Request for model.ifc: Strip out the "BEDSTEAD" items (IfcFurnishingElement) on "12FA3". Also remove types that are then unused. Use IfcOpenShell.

First a look at what the model holds.

```python
import ifcopenshell
import ifcopenshell.util.element

model = ifcopenshell.open("model.ifc")
print(model.schema)
storey = next(s for s in model.by_type("IfcBuildingStorey") if s.Name == "12FA3")
furniture = [e for e in ifcopenshell.util.element.get_decomposition(storey) if e.is_a("IfcFurnishingElement")]
seen = {}
for e in furniture:
    element_type = ifcopenshell.util.element.get_type(e)
    name = element_type.Name if element_type not in (None, e) else None
    seen[name] = seen.get(name, 0) + 1
for name, count in sorted(seen.items(), key=str):
    print(count, "x", name)
```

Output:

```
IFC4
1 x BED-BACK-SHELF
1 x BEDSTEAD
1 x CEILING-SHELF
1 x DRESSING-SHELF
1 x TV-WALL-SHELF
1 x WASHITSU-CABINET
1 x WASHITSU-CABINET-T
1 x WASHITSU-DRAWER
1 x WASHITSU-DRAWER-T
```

```python
import ifcopenshell
import ifcopenshell.api.root
import ifcopenshell.util.element

model = ifcopenshell.open("model.ifc")

storey = next(s for s in model.by_type("IfcBuildingStorey") if s.Name == "12FA3")
furniture = [e for e in ifcopenshell.util.element.get_decomposition(storey) if e.is_a("IfcFurnishingElement")]
targets = [e for e in furniture if (t := ifcopenshell.util.element.get_type(e)) not in (None, e) and t.Name == "BEDSTEAD"]
types = {ifcopenshell.util.element.get_type(e) for e in targets} - {None, *targets}

for e in targets:
    ifcopenshell.api.root.remove_product(model, product=e)
print(len(targets), "removed")

unused = [t for t in types if not ifcopenshell.util.element.get_types(t)]
for t in unused:
    ifcopenshell.api.root.remove_product(model, product=t)
print(len(unused), "unused types removed")

model.write("model_v2.ifc")
```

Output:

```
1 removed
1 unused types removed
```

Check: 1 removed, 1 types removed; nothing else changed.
